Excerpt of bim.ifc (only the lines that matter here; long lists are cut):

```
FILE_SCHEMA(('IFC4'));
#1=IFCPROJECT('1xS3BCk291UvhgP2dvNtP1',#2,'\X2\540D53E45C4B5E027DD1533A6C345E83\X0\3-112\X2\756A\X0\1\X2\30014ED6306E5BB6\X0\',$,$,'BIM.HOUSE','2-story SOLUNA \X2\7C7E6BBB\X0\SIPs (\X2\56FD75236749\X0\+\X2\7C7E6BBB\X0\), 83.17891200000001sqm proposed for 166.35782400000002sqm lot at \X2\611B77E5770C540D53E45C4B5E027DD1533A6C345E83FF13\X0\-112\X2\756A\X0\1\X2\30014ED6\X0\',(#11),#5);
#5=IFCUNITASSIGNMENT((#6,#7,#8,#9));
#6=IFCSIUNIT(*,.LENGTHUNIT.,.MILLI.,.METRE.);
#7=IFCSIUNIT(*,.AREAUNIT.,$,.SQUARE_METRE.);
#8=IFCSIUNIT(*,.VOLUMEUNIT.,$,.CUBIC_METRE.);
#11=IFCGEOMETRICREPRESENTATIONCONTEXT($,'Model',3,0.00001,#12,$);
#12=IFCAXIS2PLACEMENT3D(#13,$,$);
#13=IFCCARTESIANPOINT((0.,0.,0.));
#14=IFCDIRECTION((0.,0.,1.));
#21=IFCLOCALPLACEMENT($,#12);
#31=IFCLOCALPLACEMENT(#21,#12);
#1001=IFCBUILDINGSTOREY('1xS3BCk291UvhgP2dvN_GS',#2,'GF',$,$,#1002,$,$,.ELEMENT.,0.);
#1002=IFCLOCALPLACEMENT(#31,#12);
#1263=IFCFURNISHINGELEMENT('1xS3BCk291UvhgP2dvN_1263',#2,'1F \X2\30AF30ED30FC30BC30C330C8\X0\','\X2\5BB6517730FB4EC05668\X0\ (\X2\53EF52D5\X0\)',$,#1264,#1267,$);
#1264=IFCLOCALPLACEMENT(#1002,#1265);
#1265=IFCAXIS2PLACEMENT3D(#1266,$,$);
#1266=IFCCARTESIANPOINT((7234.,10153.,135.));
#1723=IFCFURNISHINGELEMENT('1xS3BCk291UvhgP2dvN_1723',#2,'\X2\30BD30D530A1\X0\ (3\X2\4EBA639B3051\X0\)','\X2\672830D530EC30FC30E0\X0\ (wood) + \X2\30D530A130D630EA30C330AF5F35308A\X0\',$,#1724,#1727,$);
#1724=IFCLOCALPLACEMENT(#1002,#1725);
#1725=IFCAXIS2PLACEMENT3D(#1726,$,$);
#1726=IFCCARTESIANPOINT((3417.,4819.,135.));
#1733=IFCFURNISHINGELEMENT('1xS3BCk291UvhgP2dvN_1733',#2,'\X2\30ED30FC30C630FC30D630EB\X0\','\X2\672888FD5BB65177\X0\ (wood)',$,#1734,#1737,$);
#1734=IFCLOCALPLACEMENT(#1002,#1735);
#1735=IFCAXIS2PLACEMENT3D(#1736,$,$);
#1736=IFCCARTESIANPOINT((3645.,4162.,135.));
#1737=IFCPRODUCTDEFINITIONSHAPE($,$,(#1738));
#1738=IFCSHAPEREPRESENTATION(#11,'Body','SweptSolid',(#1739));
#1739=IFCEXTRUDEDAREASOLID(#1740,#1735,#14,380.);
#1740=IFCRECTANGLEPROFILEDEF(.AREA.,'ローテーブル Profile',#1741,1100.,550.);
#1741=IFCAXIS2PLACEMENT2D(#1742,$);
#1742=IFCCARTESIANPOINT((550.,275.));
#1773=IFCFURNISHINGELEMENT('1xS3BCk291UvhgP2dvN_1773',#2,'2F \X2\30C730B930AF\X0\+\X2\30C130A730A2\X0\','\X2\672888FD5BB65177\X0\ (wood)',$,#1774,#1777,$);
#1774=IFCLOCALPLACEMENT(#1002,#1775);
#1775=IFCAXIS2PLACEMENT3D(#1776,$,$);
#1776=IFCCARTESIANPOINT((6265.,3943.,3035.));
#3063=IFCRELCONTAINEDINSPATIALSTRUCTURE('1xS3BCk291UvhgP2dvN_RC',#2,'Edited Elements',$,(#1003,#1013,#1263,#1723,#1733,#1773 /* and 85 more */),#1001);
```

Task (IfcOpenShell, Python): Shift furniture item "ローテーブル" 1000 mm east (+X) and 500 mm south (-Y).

```python
import ifcopenshell
import ifcopenshell.api.geometry
import ifcopenshell.util.placement
import ifcopenshell.util.unit

model = ifcopenshell.open("bim.ifc")
unit_scale = ifcopenshell.util.unit.calculate_unit_scale(model)

item = model.by_guid("1xS3BCk291UvhgP2dvN_1733")
matrix = ifcopenshell.util.placement.get_local_placement(item.ObjectPlacement)
matrix[0, 3] += 1 / unit_scale
matrix[1, 3] -= 0.5 / unit_scale
ifcopenshell.api.geometry.edit_object_placement(model, product=item, matrix=matrix, is_si=False)

print(ifcopenshell.util.placement.get_local_placement(item.ObjectPlacement).round(3) + 0.0)

model.write("bim_updated.ifc")
```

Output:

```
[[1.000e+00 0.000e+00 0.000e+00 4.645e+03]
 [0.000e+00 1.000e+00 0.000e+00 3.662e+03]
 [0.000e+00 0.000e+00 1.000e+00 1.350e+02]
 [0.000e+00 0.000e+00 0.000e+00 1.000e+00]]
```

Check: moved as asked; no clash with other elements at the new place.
